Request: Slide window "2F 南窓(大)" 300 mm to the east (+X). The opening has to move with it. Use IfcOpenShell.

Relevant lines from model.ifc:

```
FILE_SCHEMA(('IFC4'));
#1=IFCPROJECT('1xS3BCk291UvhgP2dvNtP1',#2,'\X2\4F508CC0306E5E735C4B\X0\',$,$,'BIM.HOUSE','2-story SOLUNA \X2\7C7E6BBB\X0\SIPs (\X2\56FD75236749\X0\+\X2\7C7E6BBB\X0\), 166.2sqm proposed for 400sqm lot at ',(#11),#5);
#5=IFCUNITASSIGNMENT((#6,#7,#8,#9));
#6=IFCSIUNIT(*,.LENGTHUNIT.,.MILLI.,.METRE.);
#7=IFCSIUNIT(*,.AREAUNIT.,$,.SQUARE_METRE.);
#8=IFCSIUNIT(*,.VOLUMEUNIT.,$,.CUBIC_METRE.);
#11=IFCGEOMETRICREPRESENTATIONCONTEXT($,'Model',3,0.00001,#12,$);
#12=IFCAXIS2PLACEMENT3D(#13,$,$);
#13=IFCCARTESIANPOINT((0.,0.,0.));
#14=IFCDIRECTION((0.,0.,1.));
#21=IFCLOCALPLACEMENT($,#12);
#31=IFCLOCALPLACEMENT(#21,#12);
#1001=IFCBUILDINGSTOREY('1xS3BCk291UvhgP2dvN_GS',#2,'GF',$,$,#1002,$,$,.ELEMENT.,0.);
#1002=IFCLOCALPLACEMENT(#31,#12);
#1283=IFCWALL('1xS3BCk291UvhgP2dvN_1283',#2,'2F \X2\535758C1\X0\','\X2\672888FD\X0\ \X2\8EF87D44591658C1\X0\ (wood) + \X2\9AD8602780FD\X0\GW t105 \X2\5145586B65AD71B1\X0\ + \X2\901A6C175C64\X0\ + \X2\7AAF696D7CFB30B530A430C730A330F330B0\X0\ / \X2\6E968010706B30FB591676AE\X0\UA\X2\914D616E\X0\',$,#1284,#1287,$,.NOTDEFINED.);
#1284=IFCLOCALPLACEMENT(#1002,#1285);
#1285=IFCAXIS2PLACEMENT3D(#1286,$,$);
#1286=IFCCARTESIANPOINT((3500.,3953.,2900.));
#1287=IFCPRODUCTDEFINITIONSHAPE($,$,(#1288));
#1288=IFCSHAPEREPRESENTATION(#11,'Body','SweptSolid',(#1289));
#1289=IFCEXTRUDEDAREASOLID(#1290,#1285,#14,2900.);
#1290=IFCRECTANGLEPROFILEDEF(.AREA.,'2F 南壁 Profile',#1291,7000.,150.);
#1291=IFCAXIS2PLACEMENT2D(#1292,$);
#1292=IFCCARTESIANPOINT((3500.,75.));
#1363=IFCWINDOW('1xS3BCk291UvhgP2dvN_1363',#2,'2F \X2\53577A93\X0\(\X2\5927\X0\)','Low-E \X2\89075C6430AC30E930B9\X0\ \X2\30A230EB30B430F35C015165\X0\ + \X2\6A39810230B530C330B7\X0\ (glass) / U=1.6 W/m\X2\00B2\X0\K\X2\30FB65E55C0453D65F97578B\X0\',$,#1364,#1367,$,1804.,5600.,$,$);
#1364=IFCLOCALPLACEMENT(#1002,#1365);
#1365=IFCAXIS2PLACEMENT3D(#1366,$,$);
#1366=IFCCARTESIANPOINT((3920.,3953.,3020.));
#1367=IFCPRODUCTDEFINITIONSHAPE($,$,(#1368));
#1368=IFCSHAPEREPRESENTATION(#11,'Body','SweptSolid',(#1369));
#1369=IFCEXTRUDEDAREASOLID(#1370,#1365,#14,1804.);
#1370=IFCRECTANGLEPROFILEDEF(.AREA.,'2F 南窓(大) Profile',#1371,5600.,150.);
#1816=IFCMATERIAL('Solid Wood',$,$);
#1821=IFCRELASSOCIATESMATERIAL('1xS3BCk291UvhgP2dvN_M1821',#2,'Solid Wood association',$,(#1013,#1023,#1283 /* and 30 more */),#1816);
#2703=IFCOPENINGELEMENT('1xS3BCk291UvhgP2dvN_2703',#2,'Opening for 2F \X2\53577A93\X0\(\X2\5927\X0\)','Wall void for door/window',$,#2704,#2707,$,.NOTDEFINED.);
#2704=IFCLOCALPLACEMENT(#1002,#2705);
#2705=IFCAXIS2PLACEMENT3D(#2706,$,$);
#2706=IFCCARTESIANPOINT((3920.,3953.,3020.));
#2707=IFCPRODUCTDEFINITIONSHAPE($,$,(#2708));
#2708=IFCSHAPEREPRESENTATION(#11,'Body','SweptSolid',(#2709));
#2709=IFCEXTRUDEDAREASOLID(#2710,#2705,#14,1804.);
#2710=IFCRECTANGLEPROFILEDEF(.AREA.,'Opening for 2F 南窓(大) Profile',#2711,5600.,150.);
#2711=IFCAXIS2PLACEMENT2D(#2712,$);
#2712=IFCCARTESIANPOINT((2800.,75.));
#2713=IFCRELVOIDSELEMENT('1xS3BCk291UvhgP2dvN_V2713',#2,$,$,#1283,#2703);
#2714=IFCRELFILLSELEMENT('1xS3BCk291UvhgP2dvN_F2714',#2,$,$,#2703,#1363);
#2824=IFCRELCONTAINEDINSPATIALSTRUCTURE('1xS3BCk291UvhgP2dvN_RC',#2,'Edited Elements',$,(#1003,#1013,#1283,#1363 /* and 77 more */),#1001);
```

```python
import ifcopenshell
import ifcopenshell.api.geometry
import ifcopenshell.util.placement
import ifcopenshell.util.unit

model = ifcopenshell.open("model.ifc")
unit_scale = ifcopenshell.util.unit.calculate_unit_scale(model)

window = model.by_id(1363)
opening = window.FillsVoids[0].RelatingOpeningElement
wall = opening.VoidsElements[0].RelatingBuildingElement

wall_matrix = ifcopenshell.util.placement.get_local_placement(wall.ObjectPlacement)
shift = wall_matrix[:3, 0] * 0.3 / unit_scale
before = ifcopenshell.util.placement.get_local_placement(window.ObjectPlacement)[:3, 3].copy()

# The window is not placed relative to its opening, so move both.
for product in (opening, window):
    matrix = ifcopenshell.util.placement.get_local_placement(product.ObjectPlacement)
    matrix[:3, 3] += shift
    ifcopenshell.api.geometry.edit_object_placement(model, product=product, matrix=matrix, is_si=False)

after = ifcopenshell.util.placement.get_local_placement(window.ObjectPlacement)[:3, 3]
print("window moved by", (after - before).round(3) + 0.0)

model.write("model_updated.ifc")
```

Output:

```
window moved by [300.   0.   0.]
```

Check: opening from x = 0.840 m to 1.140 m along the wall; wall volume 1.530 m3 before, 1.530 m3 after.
